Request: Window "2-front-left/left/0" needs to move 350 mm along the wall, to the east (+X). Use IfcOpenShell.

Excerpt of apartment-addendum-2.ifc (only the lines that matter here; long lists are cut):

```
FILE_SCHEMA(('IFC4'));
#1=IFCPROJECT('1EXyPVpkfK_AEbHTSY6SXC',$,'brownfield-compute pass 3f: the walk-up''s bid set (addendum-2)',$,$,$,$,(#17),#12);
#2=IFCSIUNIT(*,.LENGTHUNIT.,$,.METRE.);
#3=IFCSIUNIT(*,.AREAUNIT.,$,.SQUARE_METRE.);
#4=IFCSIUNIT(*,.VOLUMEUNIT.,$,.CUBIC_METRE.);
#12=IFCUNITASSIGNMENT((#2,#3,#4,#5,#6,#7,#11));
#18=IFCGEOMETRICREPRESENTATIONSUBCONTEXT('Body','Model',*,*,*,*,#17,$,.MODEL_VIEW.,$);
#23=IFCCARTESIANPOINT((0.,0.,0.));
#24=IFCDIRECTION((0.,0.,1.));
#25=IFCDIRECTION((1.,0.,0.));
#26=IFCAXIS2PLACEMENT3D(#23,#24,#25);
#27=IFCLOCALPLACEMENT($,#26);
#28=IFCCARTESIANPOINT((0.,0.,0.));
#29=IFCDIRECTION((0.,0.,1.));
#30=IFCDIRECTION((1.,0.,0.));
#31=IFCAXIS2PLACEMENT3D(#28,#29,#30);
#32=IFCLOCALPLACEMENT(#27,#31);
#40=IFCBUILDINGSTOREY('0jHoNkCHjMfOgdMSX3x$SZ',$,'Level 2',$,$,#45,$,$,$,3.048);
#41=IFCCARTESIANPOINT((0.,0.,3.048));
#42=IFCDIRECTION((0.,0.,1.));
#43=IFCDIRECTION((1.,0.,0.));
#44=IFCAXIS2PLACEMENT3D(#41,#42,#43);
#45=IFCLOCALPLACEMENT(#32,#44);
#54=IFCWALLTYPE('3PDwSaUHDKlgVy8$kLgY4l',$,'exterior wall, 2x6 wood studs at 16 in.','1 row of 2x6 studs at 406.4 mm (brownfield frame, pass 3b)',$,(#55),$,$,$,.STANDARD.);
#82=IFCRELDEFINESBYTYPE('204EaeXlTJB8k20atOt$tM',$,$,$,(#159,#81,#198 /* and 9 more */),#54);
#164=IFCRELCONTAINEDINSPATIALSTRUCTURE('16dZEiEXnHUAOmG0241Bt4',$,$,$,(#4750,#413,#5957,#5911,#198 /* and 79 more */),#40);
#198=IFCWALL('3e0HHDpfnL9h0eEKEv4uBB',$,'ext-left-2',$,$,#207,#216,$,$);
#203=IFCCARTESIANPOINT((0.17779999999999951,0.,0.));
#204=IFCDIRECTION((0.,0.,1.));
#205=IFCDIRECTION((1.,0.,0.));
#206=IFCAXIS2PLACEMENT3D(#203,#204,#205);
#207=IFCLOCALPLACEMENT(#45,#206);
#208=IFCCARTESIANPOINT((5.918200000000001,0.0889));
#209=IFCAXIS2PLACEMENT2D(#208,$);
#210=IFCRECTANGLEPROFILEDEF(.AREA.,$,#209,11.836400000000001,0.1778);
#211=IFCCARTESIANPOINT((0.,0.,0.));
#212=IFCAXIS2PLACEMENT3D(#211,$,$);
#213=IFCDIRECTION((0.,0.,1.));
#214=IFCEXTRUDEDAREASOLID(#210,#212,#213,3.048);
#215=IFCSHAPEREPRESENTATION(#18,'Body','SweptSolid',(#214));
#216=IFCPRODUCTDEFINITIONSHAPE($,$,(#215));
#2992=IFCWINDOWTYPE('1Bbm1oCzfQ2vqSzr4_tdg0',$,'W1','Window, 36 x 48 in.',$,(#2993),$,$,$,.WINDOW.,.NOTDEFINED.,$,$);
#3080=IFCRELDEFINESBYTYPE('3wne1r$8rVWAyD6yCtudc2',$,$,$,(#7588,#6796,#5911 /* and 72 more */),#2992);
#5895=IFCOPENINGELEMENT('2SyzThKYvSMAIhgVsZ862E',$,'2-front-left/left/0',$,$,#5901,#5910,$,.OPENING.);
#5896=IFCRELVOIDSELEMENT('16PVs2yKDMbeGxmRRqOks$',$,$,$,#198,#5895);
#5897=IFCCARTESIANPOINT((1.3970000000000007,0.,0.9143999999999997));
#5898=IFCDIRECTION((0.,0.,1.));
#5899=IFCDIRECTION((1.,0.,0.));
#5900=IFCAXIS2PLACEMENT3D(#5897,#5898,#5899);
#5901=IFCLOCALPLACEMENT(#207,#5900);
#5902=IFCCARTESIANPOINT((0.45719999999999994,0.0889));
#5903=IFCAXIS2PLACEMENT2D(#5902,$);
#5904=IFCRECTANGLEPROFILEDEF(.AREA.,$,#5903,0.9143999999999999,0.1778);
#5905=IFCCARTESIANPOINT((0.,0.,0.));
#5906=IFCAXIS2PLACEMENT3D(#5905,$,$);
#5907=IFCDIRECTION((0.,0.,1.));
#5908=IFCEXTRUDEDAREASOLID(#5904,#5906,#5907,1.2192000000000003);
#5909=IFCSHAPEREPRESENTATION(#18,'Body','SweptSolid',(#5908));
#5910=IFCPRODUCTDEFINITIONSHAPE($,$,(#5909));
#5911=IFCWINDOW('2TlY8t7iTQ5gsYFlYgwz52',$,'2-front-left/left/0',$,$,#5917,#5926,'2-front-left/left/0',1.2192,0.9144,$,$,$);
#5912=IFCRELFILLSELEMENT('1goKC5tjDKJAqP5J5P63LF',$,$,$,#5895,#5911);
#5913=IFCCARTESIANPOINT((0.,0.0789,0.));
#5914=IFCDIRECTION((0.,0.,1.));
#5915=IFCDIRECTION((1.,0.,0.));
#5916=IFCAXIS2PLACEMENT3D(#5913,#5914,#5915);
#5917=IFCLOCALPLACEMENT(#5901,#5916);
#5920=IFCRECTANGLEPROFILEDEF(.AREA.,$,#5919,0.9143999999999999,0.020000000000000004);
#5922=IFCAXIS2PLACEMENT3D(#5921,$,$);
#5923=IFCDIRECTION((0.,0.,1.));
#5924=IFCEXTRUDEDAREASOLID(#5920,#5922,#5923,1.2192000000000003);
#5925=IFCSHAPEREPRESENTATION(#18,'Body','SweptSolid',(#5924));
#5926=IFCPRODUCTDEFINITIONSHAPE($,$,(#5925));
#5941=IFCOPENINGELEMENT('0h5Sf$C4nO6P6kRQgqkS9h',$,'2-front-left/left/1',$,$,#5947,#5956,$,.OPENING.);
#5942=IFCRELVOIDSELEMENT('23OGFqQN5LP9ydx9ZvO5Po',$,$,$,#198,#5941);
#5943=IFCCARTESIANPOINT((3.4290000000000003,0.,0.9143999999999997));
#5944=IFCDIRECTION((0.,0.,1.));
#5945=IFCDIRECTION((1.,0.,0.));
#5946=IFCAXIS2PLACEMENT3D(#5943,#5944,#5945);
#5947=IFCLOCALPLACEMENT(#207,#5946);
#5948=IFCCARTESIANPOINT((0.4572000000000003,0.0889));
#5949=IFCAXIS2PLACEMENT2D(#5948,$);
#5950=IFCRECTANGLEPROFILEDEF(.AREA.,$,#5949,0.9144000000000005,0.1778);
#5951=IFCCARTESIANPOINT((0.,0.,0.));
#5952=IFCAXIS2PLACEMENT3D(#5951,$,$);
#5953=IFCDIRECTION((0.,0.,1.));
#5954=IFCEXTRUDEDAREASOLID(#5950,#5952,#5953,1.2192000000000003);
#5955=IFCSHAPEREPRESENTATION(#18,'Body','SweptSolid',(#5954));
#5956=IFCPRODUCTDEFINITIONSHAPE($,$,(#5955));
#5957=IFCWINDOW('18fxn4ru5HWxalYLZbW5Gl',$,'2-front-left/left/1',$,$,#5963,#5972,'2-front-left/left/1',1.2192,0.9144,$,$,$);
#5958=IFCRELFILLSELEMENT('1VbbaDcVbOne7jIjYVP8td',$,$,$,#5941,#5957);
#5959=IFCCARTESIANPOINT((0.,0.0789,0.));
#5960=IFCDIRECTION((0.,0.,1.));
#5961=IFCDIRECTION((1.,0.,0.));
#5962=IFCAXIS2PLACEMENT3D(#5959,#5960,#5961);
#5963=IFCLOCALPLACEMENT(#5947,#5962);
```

```python
import ifcopenshell
import ifcopenshell.api.geometry
import ifcopenshell.util.placement
import ifcopenshell.util.unit

model = ifcopenshell.open("apartment-addendum-2.ifc")
unit_scale = ifcopenshell.util.unit.calculate_unit_scale(model)

window = model.by_guid("2TlY8t7iTQ5gsYFlYgwz52")
opening = window.FillsVoids[0].RelatingOpeningElement
wall = opening.VoidsElements[0].RelatingBuildingElement

wall_matrix = ifcopenshell.util.placement.get_local_placement(wall.ObjectPlacement)
shift = wall_matrix[:3, 0] * 0.35 / unit_scale
before = ifcopenshell.util.placement.get_local_placement(window.ObjectPlacement)[:3, 3].copy()

# The window is placed relative to its opening, so it follows when the opening moves.
matrix = ifcopenshell.util.placement.get_local_placement(opening.ObjectPlacement)
matrix[:3, 3] += shift
ifcopenshell.api.geometry.edit_object_placement(
    model, product=opening, matrix=matrix, is_si=False, should_transform_children=True
)

after = ifcopenshell.util.placement.get_local_placement(window.ObjectPlacement)[:3, 3]
print("window moved by", (after - before).round(3) + 0.0)

model.write("apartment-addendum-2_edited.ifc")
```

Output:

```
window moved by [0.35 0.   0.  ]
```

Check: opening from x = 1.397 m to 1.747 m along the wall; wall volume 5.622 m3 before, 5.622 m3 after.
